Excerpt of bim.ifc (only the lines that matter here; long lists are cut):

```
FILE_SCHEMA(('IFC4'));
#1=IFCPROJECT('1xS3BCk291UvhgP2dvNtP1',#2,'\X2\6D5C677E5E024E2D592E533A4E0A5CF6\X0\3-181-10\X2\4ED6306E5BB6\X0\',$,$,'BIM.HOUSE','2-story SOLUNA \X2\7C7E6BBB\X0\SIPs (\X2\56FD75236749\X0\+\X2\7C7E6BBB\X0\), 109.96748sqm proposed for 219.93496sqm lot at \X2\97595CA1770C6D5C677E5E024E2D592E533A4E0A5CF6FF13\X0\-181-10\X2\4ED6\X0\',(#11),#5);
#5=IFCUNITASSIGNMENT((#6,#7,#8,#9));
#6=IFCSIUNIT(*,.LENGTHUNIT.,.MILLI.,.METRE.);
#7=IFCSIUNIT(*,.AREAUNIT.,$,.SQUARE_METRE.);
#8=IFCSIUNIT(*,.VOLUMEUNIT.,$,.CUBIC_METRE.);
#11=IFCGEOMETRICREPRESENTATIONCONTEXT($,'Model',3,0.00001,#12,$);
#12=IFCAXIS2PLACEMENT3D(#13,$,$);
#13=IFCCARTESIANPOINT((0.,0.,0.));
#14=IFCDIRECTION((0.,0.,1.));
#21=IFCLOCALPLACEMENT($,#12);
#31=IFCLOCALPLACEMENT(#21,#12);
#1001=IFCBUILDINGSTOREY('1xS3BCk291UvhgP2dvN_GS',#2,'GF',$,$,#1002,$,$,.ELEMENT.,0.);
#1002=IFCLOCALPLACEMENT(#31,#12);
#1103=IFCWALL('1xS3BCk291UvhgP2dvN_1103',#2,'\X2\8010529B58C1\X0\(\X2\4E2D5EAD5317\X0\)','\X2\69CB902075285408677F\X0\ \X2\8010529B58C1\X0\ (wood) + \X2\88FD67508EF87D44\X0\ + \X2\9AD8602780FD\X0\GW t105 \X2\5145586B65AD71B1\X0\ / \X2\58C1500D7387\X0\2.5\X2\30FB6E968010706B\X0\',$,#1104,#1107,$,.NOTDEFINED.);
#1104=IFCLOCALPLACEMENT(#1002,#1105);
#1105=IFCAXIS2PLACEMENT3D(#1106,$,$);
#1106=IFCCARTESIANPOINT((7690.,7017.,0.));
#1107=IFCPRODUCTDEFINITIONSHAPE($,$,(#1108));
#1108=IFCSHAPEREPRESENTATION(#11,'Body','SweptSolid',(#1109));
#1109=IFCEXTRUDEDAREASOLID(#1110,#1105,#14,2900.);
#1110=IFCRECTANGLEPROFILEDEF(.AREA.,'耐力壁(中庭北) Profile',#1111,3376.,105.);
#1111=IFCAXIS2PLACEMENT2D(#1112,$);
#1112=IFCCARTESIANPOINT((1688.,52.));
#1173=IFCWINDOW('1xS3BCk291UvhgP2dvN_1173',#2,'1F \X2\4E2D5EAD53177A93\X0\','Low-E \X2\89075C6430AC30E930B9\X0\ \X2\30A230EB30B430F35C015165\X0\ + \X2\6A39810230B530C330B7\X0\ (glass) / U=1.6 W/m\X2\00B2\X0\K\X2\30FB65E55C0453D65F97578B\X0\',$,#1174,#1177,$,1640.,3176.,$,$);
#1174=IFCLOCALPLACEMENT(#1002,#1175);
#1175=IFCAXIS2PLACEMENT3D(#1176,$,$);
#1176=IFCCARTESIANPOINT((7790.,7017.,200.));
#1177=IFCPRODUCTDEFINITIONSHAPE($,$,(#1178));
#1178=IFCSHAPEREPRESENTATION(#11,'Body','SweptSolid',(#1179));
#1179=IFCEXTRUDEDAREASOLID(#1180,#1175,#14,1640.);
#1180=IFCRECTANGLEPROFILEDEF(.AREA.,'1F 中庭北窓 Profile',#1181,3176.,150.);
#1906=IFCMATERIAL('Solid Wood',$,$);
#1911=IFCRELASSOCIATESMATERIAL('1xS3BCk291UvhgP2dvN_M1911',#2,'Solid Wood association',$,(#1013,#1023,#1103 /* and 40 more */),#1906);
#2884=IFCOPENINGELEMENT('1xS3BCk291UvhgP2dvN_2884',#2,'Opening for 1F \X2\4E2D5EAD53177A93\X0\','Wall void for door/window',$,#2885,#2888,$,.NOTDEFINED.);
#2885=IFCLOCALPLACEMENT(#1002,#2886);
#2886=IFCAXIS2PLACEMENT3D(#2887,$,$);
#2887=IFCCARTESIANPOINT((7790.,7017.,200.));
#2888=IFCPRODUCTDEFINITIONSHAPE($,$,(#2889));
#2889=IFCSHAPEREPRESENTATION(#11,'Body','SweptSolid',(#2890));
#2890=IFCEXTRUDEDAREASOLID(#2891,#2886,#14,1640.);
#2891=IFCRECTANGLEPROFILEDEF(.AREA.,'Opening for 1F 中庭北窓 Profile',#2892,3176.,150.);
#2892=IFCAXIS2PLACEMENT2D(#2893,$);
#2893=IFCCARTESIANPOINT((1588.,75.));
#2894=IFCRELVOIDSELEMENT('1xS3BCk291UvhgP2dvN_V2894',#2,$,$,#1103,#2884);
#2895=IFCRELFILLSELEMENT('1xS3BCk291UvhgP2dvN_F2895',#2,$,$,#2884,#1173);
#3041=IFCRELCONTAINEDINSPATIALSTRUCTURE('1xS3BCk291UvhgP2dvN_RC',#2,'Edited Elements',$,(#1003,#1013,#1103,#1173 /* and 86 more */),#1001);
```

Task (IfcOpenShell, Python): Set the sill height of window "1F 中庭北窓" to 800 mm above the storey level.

```python
import numpy as np
import ifcopenshell
import ifcopenshell.api.geometry
import ifcopenshell.geom
import ifcopenshell.util.element
import ifcopenshell.util.placement
import ifcopenshell.util.shape
import ifcopenshell.util.unit

model = ifcopenshell.open("bim.ifc")
unit_scale = ifcopenshell.util.unit.calculate_unit_scale(model)

window = model.by_id(1173)
opening = window.FillsVoids[0].RelatingOpeningElement
storey = ifcopenshell.util.element.get_container(window, ifc_class="IfcBuildingStorey")
level = ifcopenshell.util.placement.get_local_placement(storey.ObjectPlacement)[2, 3]

# The opening's origin need not be at the sill, so measure its lowest point.
shape = ifcopenshell.geom.create_shape(ifcopenshell.geom.settings(), opening)
bottom = ifcopenshell.util.shape.get_shape_bottom_elevation(shape, shape.geometry) / unit_scale
dz = level + 0.8 / unit_scale - bottom

shift = np.array([0.0, 0.0, dz])
# The window is not placed relative to its opening, so move both.
for product in (opening, window):
    matrix = ifcopenshell.util.placement.get_local_placement(product.ObjectPlacement)
    matrix[:3, 3] += shift
    ifcopenshell.api.geometry.edit_object_placement(model, product=product, matrix=matrix, is_si=False)

print(f"moved by {dz * unit_scale:+.3f} m")

model.write("bim_v2.ifc")
```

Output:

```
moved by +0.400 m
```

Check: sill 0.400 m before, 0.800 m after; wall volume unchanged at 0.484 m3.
